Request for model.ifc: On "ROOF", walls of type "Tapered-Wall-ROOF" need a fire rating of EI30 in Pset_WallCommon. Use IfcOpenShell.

First a look at what the model holds.

```python
import ifcopenshell
import ifcopenshell.util.element

model = ifcopenshell.open("model.ifc")
print(model.schema)
storey = next(s for s in model.by_type("IfcBuildingStorey") if s.Name == "ROOF")
walls = [e for e in ifcopenshell.util.element.get_decomposition(storey) if e.is_a("IfcWall")]
seen = {}
for e in walls:
    element_type = ifcopenshell.util.element.get_type(e)
    key = (element_type.Name if element_type != e and element_type else None, ifcopenshell.util.element.get_pset(e, "Pset_WallCommon", "FireRating"))
    seen[key] = seen.get(key, 0) + 1
for (name, value), count in sorted(seen.items(), key=str):
    print(count, "x", name, "|", value)
```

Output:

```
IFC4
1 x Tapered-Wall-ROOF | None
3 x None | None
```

```python
import ifcopenshell
import ifcopenshell.api.pset
import ifcopenshell.util.element

model = ifcopenshell.open("model.ifc")

storey = next(s for s in model.by_type("IfcBuildingStorey") if s.Name == "ROOF")
walls = [e for e in ifcopenshell.util.element.get_decomposition(storey) if e.is_a("IfcWall")]

count = 0
for e in walls:
    element_type = ifcopenshell.util.element.get_type(e)
    if element_type in (None, e) or element_type.Name != "Tapered-Wall-ROOF":
        continue
    # add_pset returns the element's existing set when there is one.
    pset = ifcopenshell.api.pset.add_pset(model, product=e, name="Pset_WallCommon")
    ifcopenshell.api.pset.edit_pset(model, pset=pset, properties={"FireRating": "EI30"})
    count += 1

print(count, "walls updated")

model.write("model_updated.ifc")
```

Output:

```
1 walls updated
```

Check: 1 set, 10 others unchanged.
